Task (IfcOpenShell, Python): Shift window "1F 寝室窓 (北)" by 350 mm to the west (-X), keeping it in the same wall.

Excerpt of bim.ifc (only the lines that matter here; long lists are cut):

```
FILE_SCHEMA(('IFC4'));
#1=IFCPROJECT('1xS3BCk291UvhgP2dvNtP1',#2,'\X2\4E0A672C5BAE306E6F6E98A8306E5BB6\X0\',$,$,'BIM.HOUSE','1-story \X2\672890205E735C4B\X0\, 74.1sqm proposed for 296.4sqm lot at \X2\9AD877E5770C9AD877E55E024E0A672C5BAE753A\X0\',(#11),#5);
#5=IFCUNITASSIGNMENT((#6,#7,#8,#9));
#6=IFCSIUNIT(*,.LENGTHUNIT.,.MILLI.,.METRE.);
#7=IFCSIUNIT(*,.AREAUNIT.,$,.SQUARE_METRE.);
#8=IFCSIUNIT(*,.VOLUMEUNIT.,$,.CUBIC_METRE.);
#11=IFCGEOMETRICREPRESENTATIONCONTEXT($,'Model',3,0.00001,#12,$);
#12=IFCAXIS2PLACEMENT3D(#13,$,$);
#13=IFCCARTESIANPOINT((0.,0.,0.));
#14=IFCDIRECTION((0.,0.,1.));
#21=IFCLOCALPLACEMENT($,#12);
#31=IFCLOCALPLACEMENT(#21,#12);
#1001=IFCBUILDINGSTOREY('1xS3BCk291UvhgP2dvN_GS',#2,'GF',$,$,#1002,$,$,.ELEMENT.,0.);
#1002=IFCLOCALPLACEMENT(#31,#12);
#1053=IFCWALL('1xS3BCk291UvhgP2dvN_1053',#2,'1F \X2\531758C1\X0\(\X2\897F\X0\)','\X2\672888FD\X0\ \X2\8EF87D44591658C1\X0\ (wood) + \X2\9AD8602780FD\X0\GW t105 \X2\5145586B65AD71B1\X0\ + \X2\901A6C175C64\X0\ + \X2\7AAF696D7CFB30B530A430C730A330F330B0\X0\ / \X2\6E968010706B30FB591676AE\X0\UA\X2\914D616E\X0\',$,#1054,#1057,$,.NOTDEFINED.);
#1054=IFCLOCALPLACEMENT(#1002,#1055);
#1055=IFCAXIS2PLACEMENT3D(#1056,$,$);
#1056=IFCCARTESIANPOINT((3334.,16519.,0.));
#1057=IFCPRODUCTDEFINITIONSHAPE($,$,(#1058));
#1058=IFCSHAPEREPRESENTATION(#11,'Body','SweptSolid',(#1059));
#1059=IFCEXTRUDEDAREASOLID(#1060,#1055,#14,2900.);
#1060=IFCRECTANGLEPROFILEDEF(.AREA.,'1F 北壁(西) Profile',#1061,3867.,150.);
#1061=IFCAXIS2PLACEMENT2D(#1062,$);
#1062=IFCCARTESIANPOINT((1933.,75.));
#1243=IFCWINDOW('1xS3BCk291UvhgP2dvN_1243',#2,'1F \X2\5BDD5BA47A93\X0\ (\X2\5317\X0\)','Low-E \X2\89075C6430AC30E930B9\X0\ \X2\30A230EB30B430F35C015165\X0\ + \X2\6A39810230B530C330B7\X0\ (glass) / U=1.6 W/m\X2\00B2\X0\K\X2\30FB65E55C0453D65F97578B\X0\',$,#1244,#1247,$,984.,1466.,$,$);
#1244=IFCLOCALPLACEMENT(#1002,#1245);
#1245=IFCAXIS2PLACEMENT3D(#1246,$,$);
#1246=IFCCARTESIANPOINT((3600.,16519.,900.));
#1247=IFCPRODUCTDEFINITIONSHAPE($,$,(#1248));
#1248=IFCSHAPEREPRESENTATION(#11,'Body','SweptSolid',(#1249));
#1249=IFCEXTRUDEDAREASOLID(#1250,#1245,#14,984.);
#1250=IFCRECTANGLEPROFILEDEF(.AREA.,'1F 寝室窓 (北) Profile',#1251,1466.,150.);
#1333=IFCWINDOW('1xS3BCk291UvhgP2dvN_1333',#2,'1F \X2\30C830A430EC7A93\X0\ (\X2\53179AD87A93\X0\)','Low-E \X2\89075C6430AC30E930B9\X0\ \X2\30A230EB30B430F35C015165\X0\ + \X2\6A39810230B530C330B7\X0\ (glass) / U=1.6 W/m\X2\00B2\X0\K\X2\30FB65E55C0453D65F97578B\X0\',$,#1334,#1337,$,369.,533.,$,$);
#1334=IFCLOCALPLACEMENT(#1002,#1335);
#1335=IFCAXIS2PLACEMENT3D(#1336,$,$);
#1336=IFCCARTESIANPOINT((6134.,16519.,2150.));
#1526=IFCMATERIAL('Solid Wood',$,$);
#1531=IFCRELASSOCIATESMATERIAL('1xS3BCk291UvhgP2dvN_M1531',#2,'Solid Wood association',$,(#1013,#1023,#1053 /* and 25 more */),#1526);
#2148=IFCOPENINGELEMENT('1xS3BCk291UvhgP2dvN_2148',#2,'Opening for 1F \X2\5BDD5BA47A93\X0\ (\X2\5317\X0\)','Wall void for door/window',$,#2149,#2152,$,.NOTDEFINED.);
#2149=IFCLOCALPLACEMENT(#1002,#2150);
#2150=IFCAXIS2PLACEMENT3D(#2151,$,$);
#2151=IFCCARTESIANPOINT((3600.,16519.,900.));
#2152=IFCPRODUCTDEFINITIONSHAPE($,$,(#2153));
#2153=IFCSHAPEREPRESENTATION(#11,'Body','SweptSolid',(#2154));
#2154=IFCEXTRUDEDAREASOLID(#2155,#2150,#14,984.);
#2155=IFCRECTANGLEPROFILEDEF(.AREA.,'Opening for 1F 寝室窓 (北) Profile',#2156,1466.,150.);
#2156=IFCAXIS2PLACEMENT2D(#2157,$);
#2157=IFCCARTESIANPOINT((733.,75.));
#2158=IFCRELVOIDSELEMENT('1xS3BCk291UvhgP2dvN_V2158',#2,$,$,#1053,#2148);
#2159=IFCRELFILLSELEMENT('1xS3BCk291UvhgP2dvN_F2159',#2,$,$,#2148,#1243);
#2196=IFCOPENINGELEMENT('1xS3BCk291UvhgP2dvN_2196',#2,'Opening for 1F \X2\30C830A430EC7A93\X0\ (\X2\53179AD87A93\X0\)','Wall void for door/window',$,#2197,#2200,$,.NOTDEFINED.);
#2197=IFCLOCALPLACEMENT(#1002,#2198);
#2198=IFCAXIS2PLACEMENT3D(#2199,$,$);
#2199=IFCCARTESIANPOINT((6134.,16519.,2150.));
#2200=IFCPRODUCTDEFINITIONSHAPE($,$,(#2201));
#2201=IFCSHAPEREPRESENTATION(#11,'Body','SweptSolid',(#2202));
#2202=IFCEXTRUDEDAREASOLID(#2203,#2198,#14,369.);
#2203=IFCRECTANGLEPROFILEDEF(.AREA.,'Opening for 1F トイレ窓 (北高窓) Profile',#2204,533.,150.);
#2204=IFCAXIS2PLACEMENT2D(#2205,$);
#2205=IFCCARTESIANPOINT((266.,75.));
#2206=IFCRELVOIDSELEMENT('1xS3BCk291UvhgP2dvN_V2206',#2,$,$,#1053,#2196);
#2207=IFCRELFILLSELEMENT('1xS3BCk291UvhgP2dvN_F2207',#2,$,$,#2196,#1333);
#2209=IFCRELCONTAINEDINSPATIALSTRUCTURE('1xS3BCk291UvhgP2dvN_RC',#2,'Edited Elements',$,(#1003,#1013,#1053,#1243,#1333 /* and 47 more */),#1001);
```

```python
import ifcopenshell
import ifcopenshell.api.geometry
import ifcopenshell.util.placement
import ifcopenshell.util.unit

model = ifcopenshell.open("bim.ifc")
unit_scale = ifcopenshell.util.unit.calculate_unit_scale(model)

window = model.by_guid("1xS3BCk291UvhgP2dvN_1243")
opening = window.FillsVoids[0].RelatingOpeningElement
wall = opening.VoidsElements[0].RelatingBuildingElement

wall_matrix = ifcopenshell.util.placement.get_local_placement(wall.ObjectPlacement)
shift = wall_matrix[:3, 0] * -0.35 / unit_scale
before = ifcopenshell.util.placement.get_local_placement(window.ObjectPlacement)[:3, 3].copy()

# The window is not placed relative to its opening, so move both.
for product in (opening, window):
    matrix = ifcopenshell.util.placement.get_local_placement(product.ObjectPlacement)
    matrix[:3, 3] += shift
    ifcopenshell.api.geometry.edit_object_placement(model, product=product, matrix=matrix, is_si=False)

after = ifcopenshell.util.placement.get_local_placement(window.ObjectPlacement)[:3, 3]
print("window moved by", (after - before).round(3) + 0.0)

model.write("bim_edited.ifc")
```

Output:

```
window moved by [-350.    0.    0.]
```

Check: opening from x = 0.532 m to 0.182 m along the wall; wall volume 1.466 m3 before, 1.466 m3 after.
